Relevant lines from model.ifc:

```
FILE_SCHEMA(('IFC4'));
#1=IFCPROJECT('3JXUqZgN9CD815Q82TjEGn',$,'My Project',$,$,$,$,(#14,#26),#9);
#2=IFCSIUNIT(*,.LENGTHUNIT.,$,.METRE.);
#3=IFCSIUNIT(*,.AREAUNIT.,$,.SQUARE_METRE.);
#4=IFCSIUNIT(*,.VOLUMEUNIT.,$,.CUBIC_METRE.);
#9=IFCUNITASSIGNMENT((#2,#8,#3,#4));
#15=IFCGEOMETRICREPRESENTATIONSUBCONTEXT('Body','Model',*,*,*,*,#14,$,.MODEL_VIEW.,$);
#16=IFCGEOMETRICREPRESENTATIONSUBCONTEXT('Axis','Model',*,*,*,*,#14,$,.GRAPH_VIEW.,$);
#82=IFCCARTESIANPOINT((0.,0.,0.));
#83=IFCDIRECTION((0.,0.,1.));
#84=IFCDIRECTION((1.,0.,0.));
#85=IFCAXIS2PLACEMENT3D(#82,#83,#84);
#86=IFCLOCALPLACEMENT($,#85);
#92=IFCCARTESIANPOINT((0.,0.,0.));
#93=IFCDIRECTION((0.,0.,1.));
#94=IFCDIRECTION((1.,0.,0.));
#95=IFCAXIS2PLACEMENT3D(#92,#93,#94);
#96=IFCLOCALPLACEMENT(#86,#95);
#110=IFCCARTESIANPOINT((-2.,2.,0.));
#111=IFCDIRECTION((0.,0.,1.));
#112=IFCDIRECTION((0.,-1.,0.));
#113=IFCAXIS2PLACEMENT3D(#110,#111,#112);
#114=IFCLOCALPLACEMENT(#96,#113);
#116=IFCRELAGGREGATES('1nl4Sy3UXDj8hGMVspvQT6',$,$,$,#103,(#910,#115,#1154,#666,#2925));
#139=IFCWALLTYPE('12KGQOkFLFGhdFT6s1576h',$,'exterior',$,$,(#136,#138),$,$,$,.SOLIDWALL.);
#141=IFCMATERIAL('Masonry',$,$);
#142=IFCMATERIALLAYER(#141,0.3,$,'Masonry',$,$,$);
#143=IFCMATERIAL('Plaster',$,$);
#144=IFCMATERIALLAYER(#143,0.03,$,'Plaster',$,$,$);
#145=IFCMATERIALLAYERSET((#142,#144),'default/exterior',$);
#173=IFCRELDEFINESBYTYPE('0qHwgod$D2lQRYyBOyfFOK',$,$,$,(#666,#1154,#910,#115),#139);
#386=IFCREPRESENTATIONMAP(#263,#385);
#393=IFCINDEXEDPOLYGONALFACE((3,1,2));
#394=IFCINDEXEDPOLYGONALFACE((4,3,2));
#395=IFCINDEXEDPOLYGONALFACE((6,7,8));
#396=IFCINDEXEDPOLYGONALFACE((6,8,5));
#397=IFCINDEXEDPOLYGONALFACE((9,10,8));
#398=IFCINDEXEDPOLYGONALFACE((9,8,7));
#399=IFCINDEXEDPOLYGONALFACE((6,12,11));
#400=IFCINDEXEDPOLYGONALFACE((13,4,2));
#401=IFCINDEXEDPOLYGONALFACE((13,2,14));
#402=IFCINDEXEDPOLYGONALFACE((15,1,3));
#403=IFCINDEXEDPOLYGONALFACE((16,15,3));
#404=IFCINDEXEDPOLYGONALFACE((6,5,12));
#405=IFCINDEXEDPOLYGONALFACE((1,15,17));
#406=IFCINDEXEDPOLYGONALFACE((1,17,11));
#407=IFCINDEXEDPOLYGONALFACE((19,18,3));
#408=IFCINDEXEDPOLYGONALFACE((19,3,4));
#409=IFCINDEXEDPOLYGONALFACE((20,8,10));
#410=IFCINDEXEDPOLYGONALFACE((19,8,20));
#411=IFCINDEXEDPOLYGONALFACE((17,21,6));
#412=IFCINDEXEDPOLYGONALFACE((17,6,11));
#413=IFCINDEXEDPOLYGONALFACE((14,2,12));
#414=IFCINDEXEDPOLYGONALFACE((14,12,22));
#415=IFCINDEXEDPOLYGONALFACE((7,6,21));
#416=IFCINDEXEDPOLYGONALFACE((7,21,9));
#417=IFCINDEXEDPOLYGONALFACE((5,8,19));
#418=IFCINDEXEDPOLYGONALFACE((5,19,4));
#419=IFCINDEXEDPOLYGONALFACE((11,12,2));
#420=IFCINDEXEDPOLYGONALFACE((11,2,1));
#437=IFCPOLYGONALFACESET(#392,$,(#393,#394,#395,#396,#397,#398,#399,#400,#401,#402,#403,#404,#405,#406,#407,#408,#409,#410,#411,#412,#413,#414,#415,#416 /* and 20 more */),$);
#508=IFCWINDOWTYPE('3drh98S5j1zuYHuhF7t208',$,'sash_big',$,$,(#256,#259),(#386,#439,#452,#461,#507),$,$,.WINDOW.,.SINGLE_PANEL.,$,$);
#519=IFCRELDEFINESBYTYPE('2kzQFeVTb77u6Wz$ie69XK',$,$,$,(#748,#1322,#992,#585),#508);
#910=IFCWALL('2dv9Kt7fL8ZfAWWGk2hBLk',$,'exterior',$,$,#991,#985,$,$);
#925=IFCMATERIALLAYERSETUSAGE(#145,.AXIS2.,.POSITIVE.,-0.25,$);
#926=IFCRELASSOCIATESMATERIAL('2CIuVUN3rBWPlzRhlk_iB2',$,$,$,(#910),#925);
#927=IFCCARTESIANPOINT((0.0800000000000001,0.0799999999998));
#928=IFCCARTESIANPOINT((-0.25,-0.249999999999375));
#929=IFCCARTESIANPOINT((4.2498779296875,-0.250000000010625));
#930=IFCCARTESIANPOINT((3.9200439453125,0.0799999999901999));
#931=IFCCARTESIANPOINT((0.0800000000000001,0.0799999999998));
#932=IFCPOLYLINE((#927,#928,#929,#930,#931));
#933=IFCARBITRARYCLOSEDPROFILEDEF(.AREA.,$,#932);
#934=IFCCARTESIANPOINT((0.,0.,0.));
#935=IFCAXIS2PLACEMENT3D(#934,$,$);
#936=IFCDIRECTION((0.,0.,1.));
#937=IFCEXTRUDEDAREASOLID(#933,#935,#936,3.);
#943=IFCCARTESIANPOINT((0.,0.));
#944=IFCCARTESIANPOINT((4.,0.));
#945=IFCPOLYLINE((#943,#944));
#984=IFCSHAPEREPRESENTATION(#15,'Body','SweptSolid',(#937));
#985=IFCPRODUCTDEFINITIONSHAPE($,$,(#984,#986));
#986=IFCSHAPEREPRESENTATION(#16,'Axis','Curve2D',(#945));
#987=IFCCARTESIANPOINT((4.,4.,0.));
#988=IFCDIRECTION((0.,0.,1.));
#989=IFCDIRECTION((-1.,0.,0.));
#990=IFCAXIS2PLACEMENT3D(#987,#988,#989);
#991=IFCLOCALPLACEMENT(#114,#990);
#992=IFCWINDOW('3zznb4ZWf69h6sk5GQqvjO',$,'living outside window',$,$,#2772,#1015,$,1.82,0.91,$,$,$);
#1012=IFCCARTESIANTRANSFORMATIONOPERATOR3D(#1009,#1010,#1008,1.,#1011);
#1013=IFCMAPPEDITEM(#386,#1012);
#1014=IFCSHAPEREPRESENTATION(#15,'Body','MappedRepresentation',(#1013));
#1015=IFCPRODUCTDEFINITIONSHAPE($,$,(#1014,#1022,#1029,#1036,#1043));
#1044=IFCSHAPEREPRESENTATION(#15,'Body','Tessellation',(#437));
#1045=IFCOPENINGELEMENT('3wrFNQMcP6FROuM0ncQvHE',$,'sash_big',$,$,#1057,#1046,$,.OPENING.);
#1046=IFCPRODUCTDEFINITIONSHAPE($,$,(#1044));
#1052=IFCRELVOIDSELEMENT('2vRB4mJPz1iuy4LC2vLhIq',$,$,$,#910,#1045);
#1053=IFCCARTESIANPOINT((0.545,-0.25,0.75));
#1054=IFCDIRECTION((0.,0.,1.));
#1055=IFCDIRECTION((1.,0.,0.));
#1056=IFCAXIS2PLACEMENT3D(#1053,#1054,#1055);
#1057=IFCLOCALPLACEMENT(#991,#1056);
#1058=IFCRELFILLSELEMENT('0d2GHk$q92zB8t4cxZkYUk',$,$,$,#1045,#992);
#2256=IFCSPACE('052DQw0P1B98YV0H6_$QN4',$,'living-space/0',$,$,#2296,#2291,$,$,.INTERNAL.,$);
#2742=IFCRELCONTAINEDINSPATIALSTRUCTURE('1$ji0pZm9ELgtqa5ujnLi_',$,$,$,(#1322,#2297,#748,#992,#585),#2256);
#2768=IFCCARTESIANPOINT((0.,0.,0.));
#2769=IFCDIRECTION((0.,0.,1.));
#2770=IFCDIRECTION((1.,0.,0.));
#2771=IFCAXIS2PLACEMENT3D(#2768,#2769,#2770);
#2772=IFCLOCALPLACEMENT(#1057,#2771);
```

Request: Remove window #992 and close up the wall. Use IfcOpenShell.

```python
import ifcopenshell
import ifcopenshell.api.feature
import ifcopenshell.api.root
import ifcopenshell.geom
import ifcopenshell.util.shape

model = ifcopenshell.open("model.ifc")
settings = ifcopenshell.geom.settings()


def volume(element):
    """Net volume in cubic metres, openings subtracted."""
    shape = ifcopenshell.geom.create_shape(settings, element)
    return ifcopenshell.util.shape.get_volume(shape.geometry)


window = model.by_guid("3zznb4ZWf69h6sk5GQqvjO")
opening = window.FillsVoids[0].RelatingOpeningElement
wall = opening.VoidsElements[0].RelatingBuildingElement
before = volume(wall)

ifcopenshell.api.root.remove_product(model, product=window)
ifcopenshell.api.feature.remove_feature(model, feature=opening)

after = volume(wall)

print(f"wall volume {before:.3f} -> {after:.3f} m3")

model.write("model_updated.ifc")
```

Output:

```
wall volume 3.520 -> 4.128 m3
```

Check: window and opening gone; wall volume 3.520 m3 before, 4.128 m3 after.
